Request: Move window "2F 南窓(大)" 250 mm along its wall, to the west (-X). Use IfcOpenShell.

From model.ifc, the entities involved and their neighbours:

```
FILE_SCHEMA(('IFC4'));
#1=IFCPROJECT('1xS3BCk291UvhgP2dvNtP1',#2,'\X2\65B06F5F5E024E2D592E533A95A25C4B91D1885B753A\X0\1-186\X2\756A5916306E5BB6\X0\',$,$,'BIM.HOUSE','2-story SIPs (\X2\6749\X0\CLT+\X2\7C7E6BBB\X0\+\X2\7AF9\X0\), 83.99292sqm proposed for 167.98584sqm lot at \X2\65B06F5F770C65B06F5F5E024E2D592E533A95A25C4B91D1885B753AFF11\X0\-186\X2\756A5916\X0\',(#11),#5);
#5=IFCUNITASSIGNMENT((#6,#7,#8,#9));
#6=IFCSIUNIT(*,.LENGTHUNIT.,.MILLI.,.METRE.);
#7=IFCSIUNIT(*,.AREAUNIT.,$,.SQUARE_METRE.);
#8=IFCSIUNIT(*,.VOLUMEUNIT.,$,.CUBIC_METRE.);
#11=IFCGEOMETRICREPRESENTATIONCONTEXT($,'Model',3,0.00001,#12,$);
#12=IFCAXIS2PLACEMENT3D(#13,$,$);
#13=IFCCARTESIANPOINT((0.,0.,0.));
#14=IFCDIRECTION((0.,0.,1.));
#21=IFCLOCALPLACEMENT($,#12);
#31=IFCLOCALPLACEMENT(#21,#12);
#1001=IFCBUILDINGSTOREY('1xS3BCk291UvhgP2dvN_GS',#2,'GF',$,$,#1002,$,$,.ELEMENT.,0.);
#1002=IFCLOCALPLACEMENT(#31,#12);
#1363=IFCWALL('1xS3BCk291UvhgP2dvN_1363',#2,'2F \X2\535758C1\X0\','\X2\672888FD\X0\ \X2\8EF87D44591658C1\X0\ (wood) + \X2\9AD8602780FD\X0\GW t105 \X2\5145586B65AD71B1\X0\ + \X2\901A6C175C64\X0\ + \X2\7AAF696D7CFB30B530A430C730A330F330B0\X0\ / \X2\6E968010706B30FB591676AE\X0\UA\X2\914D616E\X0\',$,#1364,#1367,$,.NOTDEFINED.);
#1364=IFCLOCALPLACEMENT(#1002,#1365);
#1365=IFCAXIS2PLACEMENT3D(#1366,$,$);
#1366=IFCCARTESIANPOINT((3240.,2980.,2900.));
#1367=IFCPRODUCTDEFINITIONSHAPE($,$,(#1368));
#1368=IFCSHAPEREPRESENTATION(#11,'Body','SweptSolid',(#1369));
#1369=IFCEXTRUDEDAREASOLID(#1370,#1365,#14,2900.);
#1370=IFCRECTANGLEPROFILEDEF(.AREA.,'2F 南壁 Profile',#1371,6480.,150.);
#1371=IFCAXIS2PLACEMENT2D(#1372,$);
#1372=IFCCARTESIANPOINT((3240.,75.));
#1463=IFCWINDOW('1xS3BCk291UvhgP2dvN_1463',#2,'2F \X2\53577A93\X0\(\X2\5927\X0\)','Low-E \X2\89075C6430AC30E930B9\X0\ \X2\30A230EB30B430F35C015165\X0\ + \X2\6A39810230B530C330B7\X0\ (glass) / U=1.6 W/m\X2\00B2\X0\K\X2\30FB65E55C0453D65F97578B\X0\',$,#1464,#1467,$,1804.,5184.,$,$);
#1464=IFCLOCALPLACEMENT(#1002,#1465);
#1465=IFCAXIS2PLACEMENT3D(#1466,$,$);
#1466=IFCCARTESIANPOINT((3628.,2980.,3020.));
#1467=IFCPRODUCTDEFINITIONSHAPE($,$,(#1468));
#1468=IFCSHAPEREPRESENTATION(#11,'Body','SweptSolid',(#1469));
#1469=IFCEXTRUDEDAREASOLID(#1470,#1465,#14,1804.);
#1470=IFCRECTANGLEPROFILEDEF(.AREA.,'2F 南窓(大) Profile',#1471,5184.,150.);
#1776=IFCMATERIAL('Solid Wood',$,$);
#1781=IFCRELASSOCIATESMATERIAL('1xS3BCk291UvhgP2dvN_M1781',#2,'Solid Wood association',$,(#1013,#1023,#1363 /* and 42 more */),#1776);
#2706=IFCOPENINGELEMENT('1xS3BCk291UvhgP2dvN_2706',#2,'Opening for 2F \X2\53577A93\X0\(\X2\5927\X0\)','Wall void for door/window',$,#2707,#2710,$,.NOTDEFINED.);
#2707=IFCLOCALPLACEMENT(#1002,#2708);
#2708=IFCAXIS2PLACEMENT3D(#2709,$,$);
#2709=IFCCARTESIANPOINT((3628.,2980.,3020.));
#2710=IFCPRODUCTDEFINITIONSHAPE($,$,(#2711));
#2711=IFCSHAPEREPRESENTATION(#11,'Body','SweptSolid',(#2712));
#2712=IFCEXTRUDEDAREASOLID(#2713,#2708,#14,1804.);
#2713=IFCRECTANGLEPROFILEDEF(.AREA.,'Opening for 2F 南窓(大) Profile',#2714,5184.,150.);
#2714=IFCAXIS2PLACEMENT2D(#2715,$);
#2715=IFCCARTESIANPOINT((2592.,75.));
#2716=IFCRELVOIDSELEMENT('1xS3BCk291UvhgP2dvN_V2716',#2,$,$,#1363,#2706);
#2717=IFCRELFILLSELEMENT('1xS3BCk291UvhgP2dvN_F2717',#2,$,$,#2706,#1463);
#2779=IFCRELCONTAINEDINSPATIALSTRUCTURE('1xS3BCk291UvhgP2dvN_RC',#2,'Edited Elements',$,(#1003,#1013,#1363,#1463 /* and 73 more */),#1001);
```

```python
import ifcopenshell
import ifcopenshell.api.geometry
import ifcopenshell.util.placement
import ifcopenshell.util.unit

model = ifcopenshell.open("model.ifc")
unit_scale = ifcopenshell.util.unit.calculate_unit_scale(model)

window = model.by_guid("1xS3BCk291UvhgP2dvN_1463")
opening = window.FillsVoids[0].RelatingOpeningElement
wall = opening.VoidsElements[0].RelatingBuildingElement

wall_matrix = ifcopenshell.util.placement.get_local_placement(wall.ObjectPlacement)
shift = wall_matrix[:3, 0] * -0.25 / unit_scale
before = ifcopenshell.util.placement.get_local_placement(window.ObjectPlacement)[:3, 3].copy()

# The window is not placed relative to its opening, so move both.
for product in (opening, window):
    matrix = ifcopenshell.util.placement.get_local_placement(product.ObjectPlacement)
    matrix[:3, 3] += shift
    ifcopenshell.api.geometry.edit_object_placement(model, product=product, matrix=matrix, is_si=False)

after = ifcopenshell.util.placement.get_local_placement(window.ObjectPlacement)[:3, 3]
print("window moved by", (after - before).round(3) + 0.0)

model.write("model_edited.ifc")
```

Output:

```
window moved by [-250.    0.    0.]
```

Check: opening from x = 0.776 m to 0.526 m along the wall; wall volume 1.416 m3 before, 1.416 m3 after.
